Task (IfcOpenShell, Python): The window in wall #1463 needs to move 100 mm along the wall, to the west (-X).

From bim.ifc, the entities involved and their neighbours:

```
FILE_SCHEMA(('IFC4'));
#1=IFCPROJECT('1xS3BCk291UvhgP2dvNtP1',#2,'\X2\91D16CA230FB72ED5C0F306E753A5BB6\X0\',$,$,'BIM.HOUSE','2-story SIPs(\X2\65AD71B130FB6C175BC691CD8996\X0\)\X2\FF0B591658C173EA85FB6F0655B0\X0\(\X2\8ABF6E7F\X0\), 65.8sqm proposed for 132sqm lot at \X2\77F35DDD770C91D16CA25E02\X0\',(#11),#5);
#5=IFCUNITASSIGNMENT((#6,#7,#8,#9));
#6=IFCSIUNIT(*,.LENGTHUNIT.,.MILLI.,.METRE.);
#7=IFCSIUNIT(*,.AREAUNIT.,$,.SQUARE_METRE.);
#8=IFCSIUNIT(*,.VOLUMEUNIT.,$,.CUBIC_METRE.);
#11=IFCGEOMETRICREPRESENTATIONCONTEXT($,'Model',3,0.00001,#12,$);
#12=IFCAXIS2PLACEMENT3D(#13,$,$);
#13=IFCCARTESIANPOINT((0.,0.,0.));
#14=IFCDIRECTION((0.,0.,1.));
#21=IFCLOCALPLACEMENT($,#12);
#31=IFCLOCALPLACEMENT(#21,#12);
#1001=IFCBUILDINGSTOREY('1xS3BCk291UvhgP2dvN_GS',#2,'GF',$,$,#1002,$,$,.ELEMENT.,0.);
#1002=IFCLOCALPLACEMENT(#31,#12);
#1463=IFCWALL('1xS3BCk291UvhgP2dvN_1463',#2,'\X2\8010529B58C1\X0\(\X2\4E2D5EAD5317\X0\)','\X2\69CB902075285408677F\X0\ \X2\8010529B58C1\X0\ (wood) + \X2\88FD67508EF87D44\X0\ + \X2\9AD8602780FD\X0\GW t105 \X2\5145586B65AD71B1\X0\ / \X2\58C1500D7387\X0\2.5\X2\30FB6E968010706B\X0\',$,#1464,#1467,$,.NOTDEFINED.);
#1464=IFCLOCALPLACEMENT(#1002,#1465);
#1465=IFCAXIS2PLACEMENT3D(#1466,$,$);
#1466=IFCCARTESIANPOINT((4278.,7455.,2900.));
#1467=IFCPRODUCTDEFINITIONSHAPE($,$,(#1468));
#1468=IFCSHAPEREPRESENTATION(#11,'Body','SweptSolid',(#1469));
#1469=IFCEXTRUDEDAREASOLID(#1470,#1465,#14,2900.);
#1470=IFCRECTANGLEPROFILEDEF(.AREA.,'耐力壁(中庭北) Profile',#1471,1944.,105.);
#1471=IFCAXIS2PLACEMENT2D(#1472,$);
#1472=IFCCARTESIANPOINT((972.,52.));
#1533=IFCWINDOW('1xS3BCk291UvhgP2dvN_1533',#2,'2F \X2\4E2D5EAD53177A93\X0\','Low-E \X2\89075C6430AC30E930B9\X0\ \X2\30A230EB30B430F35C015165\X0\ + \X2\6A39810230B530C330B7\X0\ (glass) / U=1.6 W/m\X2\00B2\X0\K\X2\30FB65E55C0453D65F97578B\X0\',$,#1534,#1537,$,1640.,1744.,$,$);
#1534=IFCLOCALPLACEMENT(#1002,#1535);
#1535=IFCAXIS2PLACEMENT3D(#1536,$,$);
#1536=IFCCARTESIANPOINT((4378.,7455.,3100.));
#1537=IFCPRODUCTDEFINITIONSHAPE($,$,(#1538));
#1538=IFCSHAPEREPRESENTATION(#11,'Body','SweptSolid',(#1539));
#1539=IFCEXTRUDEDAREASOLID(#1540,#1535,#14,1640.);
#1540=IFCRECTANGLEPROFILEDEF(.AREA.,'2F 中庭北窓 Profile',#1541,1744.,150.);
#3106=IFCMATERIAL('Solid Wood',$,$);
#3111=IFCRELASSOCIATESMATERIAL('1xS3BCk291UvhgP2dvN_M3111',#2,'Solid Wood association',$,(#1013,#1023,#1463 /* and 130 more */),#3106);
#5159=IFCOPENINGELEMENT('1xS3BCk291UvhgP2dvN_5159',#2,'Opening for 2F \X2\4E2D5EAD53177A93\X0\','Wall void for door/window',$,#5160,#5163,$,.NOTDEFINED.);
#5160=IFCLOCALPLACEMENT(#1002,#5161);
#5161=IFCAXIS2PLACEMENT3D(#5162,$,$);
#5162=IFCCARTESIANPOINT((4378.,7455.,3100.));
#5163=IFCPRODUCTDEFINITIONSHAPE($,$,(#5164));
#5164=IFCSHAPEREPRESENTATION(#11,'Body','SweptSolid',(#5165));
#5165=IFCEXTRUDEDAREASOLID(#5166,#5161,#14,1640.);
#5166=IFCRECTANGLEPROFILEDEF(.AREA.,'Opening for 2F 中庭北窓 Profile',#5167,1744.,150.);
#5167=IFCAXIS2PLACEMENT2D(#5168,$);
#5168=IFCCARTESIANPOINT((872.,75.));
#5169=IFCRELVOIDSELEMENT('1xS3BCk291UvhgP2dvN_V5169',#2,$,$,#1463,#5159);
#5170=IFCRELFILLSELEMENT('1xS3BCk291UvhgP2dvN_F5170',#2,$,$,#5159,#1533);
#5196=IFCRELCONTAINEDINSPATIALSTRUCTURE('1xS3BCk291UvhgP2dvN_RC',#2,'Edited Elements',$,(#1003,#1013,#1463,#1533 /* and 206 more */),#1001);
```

```python
import ifcopenshell
import ifcopenshell.api.geometry
import ifcopenshell.util.placement
import ifcopenshell.util.unit

model = ifcopenshell.open("bim.ifc")
unit_scale = ifcopenshell.util.unit.calculate_unit_scale(model)

window = model.by_id(1533)
opening = window.FillsVoids[0].RelatingOpeningElement
wall = opening.VoidsElements[0].RelatingBuildingElement

wall_matrix = ifcopenshell.util.placement.get_local_placement(wall.ObjectPlacement)
shift = wall_matrix[:3, 0] * -0.1 / unit_scale
before = ifcopenshell.util.placement.get_local_placement(window.ObjectPlacement)[:3, 3].copy()

# The window is not placed relative to its opening, so move both.
for product in (opening, window):
    matrix = ifcopenshell.util.placement.get_local_placement(product.ObjectPlacement)
    matrix[:3, 3] += shift
    ifcopenshell.api.geometry.edit_object_placement(model, product=product, matrix=matrix, is_si=False)

after = ifcopenshell.util.placement.get_local_placement(window.ObjectPlacement)[:3, 3]
print("window moved by", (after - before).round(3) + 0.0)

model.write("bim_rev.ifc")
```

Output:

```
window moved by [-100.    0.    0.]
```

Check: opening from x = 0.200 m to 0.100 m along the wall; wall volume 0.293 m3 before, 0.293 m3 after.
